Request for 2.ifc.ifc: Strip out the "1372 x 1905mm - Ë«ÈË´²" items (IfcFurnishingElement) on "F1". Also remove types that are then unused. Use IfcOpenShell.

First a look at what the model holds.

```python
import ifcopenshell
import ifcopenshell.util.element

model = ifcopenshell.open("2.ifc.ifc")
print(model.schema)
storey = next(s for s in model.by_type("IfcBuildingStorey") if s.Name == "F1")
furniture = [e for e in ifcopenshell.util.element.get_decomposition(storey) if e.is_a("IfcFurnishingElement")]
seen = {}
for e in furniture:
    element_type = ifcopenshell.util.element.get_type(e)
    name = element_type.Name if element_type not in (None, e) else None
    seen[name] = seen.get(name, 0) + 1
for name, count in sorted(seen.items(), key=str):
    print(count, "x", name)
```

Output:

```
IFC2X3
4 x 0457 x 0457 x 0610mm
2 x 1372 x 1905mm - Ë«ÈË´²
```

```python
import ifcopenshell
import ifcopenshell.api.root
import ifcopenshell.util.element

model = ifcopenshell.open("2.ifc.ifc")

storey = next(s for s in model.by_type("IfcBuildingStorey") if s.Name == "F1")
furniture = [e for e in ifcopenshell.util.element.get_decomposition(storey) if e.is_a("IfcFurnishingElement")]
targets = [e for e in furniture if (t := ifcopenshell.util.element.get_type(e)) not in (None, e) and t.Name == "1372 x 1905mm - Ë«ÈË´²"]
types = {ifcopenshell.util.element.get_type(e) for e in targets} - {None, *targets}

for e in targets:
    ifcopenshell.api.root.remove_product(model, product=e)
print(len(targets), "removed")

unused = [t for t in types if not ifcopenshell.util.element.get_types(t)]
for t in unused:
    ifcopenshell.api.root.remove_product(model, product=t)
print(len(unused), "unused types removed")

model.write("2.ifc_rev.ifc")
```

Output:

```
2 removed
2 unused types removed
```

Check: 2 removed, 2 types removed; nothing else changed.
